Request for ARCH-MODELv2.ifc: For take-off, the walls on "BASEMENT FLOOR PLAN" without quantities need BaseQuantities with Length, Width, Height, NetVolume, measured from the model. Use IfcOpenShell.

First a look at what the model holds.

```python
import ifcopenshell
import ifcopenshell.util.element
import ifcopenshell.util.unit

model = ifcopenshell.open("ARCH-MODELv2.ifc")
print(model.schema)
for unit_type in ("LENGTHUNIT", "AREAUNIT", "VOLUMEUNIT"):
    print(unit_type, ifcopenshell.util.unit.calculate_unit_scale(model, unit_type))
storey = next(s for s in model.by_type("IfcBuildingStorey") if s.Name == "BASEMENT FLOOR PLAN")
walls = [e for e in ifcopenshell.util.element.get_decomposition(storey) if e.is_a("IfcWall")]
for e in sorted(walls, key=lambda e: e.id()):
    print(e.id(), e.is_a(), e.Name, list(ifcopenshell.util.element.get_psets(e, qtos_only=True)), sep=" | ")
```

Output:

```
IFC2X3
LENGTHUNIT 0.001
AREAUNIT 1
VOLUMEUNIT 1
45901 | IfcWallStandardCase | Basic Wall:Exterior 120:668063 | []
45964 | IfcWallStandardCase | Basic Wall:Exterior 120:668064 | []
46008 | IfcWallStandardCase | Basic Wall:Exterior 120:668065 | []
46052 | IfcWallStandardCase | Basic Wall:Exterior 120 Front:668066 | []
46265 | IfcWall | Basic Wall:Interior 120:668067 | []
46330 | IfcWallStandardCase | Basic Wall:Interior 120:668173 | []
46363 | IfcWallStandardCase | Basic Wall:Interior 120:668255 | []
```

```python
import ifcopenshell
import ifcopenshell.api.pset
import ifcopenshell.geom
import ifcopenshell.util.element
import ifcopenshell.util.shape
import ifcopenshell.util.unit

model = ifcopenshell.open("ARCH-MODELv2.ifc")
unit_scale = ifcopenshell.util.unit.calculate_unit_scale(model)
volume_scale = ifcopenshell.util.unit.calculate_unit_scale(model, "VOLUMEUNIT")
settings = ifcopenshell.geom.settings()

storey = next(s for s in model.by_type("IfcBuildingStorey") if s.Name == "BASEMENT FLOOR PLAN")
walls = [e for e in ifcopenshell.util.element.get_decomposition(storey) if e.is_a("IfcWall")]

for e in sorted(walls, key=lambda e: e.id()):
    if ifcopenshell.util.element.get_psets(e, qtos_only=True, should_inherit=False):
        continue
    # Geometry comes back in metres, in the element's own axes.
    shape = ifcopenshell.geom.create_shape(settings, e)
    values = {
        "Length": ifcopenshell.util.shape.get_x(shape.geometry) / unit_scale,
        "Width": ifcopenshell.util.shape.get_y(shape.geometry) / unit_scale,
        "Height": ifcopenshell.util.shape.get_z(shape.geometry) / unit_scale,
        "NetVolume": ifcopenshell.util.shape.get_volume(shape.geometry) / volume_scale,
    }
    qto = ifcopenshell.api.pset.add_qto(model, product=e, name="BaseQuantities")
    ifcopenshell.api.pset.edit_qto(model, qto=qto, properties=values)
    print(e.id(), {k: round(v, 3) for k, v in values.items()})

model.write("ARCH-MODELv2_rev.ifc")
```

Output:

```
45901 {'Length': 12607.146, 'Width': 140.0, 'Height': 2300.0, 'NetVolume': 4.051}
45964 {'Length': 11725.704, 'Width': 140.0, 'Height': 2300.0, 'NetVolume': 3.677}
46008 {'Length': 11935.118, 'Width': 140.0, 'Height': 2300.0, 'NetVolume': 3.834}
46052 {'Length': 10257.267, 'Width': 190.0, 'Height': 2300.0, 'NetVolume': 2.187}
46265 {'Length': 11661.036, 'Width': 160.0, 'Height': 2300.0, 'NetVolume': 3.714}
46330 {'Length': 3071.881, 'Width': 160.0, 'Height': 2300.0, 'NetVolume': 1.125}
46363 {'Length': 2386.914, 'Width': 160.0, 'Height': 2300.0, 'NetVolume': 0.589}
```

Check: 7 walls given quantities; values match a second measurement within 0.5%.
